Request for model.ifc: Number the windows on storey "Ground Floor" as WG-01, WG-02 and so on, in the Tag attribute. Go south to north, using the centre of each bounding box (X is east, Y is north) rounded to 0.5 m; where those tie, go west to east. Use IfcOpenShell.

First a look at what the model holds.

```python
import ifcopenshell
import ifcopenshell.util.element
import ifcopenshell.util.placement

model = ifcopenshell.open("model.ifc")
print(model.schema)
storey = next(s for s in model.by_type("IfcBuildingStorey") if s.Name == "Ground Floor")
windows = [e for e in ifcopenshell.util.element.get_decomposition(storey) if e.is_a("IfcWindow")]
for e in sorted(windows, key=lambda e: e.id()):
    origin = ifcopenshell.util.placement.get_local_placement(e.ObjectPlacement)[:3, 3]
    print(e.id(), e.Tag, e.Name, origin.round(2) + 0.0, sep=" | ")
```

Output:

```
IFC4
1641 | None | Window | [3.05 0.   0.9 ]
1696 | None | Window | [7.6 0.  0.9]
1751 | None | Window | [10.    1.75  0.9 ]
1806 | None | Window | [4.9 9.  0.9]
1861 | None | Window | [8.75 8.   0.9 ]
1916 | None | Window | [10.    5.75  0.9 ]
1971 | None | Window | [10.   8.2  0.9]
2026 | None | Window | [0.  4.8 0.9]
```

```python
import ifcopenshell
import ifcopenshell.geom
import ifcopenshell.util.element
import ifcopenshell.util.shape

model = ifcopenshell.open("model.ifc")
settings = ifcopenshell.geom.settings()
settings.set("use-world-coords", True)


def centre(element):
    shape = ifcopenshell.geom.create_shape(settings, element)
    return ifcopenshell.util.shape.get_bbox_centroid(shape.geometry)


storey = next(s for s in model.by_type("IfcBuildingStorey") if s.Name == "Ground Floor")
windows = [e for e in ifcopenshell.util.element.get_decomposition(storey) if e.is_a("IfcWindow")]

# Insertion points can sit at a corner or the storey origin, so sort by the geometry (in metres).
centres = {e: centre(e) for e in windows}
windows.sort(key=lambda e: (round(centres[e][1] / 0.5), centres[e][0]))

for i, e in enumerate(windows, start=1):
    number = f"WG-{i:02d}"
    e.Tag = number
    print(e.id(), number)

model.write("model_v2.ifc")
```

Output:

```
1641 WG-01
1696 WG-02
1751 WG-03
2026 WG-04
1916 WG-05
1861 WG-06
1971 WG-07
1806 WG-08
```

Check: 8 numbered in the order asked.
